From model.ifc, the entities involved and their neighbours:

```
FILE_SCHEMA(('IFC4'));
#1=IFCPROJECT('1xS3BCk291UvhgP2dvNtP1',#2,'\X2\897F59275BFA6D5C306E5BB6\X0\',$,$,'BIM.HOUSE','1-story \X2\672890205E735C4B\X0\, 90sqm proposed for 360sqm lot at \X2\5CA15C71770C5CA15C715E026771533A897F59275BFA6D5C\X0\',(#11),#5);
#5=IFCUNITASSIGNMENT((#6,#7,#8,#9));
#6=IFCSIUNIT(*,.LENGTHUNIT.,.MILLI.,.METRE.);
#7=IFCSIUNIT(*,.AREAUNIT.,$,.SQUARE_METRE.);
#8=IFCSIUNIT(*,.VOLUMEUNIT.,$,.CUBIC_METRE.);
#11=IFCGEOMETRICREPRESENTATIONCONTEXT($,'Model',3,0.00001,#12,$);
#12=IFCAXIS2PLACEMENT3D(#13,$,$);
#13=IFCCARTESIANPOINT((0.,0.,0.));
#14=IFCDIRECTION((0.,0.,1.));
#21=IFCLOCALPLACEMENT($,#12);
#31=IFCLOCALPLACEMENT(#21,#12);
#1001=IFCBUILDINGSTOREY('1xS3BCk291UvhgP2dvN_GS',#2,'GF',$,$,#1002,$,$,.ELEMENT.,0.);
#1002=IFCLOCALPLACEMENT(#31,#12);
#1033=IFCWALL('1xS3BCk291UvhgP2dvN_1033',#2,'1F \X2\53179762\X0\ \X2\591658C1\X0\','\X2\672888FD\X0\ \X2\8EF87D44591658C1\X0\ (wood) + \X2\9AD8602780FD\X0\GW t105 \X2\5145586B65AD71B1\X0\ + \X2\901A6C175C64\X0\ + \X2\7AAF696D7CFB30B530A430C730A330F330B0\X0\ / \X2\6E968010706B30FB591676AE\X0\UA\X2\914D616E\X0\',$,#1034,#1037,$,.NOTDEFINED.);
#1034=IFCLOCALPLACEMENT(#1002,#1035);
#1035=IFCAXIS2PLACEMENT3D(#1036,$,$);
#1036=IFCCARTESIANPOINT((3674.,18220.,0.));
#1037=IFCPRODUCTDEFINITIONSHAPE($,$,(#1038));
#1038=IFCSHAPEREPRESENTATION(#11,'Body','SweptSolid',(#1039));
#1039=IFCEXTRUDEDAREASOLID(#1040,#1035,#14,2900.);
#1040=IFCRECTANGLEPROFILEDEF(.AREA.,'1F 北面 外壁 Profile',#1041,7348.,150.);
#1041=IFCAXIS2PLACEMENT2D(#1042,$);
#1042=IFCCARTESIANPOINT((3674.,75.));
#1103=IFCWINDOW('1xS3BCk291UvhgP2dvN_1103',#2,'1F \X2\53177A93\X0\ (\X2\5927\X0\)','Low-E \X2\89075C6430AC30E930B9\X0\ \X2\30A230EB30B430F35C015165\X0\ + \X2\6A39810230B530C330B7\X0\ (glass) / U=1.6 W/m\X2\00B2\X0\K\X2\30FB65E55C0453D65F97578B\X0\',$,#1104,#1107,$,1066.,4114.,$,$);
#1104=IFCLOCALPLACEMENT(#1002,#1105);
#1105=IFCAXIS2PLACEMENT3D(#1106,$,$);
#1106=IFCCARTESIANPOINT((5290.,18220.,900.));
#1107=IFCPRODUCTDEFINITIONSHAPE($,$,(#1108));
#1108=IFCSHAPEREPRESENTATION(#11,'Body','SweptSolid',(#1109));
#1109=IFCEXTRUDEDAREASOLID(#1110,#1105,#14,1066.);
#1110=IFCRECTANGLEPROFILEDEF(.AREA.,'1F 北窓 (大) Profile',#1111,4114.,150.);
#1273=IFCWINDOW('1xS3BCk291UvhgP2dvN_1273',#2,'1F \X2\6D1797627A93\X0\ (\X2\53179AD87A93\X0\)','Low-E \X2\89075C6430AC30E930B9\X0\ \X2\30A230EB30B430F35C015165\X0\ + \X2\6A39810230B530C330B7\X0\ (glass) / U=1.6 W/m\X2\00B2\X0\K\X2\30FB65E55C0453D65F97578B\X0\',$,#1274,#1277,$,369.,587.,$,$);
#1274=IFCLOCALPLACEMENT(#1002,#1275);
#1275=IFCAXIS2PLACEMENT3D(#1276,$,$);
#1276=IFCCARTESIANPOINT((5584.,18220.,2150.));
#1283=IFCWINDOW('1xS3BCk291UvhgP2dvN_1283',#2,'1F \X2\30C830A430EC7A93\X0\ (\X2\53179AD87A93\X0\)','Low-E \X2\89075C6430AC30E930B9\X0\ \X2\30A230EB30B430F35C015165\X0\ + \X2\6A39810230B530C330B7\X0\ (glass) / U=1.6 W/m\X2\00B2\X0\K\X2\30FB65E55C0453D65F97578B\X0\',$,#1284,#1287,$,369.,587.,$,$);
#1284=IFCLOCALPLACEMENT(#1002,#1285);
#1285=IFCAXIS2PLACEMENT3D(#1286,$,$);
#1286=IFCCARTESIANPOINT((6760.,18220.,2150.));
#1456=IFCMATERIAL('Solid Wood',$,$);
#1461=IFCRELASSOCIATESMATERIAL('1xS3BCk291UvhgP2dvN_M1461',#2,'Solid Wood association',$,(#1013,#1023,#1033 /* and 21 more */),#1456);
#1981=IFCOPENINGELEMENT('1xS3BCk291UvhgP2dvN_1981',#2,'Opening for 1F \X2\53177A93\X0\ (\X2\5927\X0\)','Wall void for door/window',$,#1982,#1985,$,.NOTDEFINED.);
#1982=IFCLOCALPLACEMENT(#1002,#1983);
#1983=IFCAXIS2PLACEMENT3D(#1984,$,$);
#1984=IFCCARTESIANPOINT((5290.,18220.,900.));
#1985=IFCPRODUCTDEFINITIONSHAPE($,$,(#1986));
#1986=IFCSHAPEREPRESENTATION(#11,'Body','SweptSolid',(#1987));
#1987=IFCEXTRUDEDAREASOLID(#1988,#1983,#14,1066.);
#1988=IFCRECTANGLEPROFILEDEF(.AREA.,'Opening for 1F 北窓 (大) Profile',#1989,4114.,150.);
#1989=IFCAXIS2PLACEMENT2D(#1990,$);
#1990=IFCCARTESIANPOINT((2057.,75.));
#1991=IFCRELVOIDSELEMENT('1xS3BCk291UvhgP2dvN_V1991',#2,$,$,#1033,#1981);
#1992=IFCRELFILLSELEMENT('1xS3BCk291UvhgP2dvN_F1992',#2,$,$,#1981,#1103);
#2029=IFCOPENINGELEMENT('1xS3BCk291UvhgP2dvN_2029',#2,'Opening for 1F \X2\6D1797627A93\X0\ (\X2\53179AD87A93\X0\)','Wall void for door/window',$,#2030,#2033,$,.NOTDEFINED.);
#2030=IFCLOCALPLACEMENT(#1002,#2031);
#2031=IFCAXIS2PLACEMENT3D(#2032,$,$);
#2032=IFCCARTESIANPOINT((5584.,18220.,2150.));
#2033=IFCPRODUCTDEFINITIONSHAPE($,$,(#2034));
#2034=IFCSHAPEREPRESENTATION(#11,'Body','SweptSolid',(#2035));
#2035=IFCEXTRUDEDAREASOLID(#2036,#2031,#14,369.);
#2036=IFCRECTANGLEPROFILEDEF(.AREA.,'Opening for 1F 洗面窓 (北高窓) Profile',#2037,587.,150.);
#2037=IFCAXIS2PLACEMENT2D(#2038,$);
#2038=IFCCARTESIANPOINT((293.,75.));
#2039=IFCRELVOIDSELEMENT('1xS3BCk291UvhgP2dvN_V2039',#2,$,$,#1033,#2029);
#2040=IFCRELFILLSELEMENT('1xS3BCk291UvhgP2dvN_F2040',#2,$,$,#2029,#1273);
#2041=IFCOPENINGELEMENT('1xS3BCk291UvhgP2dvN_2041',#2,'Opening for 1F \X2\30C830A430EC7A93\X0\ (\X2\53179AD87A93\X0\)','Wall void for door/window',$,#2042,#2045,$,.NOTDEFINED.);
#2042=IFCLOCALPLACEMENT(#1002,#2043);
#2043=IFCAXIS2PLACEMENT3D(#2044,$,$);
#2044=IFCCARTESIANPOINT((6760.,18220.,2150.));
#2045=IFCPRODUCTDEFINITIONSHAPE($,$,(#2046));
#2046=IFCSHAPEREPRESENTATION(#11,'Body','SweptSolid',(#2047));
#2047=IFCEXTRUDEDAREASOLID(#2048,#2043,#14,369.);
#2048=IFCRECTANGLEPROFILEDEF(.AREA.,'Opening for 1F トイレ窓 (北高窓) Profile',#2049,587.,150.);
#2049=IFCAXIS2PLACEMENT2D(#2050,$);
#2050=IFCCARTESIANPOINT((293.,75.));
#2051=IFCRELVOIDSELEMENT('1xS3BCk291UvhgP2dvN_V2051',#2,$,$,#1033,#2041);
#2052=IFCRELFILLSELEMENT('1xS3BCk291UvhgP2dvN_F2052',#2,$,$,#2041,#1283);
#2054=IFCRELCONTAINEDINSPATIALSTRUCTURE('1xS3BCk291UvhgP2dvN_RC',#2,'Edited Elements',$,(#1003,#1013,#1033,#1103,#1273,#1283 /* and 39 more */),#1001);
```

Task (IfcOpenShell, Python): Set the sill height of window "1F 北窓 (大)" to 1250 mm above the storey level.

```python
import numpy as np
import ifcopenshell
import ifcopenshell.api.geometry
import ifcopenshell.geom
import ifcopenshell.util.element
import ifcopenshell.util.placement
import ifcopenshell.util.shape
import ifcopenshell.util.unit

model = ifcopenshell.open("model.ifc")
unit_scale = ifcopenshell.util.unit.calculate_unit_scale(model)

window = model.by_guid("1xS3BCk291UvhgP2dvN_1103")
opening = window.FillsVoids[0].RelatingOpeningElement
storey = ifcopenshell.util.element.get_container(window, ifc_class="IfcBuildingStorey")
level = ifcopenshell.util.placement.get_local_placement(storey.ObjectPlacement)[2, 3]

# The opening's origin need not be at the sill, so measure its lowest point.
shape = ifcopenshell.geom.create_shape(ifcopenshell.geom.settings(), opening)
bottom = ifcopenshell.util.shape.get_shape_bottom_elevation(shape, shape.geometry) / unit_scale
dz = level + 1250.0 - bottom

shift = np.array([0.0, 0.0, dz])
# The window is not placed relative to its opening, so move both.
for product in (opening, window):
    matrix = ifcopenshell.util.placement.get_local_placement(product.ObjectPlacement)
    matrix[:3, 3] += shift
    ifcopenshell.api.geometry.edit_object_placement(model, product=product, matrix=matrix, is_si=False)

print(f"moved by {dz * unit_scale:+.3f} m")

model.write("model_rev.ifc")
```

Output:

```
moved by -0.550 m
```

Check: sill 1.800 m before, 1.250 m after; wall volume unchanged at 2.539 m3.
